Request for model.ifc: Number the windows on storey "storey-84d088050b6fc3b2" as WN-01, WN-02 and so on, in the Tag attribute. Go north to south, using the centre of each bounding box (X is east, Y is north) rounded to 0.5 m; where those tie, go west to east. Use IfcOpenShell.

First a look at what the model holds.

```python
import ifcopenshell
import ifcopenshell.util.element
import ifcopenshell.util.placement

model = ifcopenshell.open("model.ifc")
print(model.schema)
storey = next(s for s in model.by_type("IfcBuildingStorey") if s.Name == "storey-84d088050b6fc3b2")
windows = [e for e in ifcopenshell.util.element.get_decomposition(storey) if e.is_a("IfcWindow")]
for e in sorted(windows, key=lambda e: e.id()):
    origin = ifcopenshell.util.placement.get_local_placement(e.ObjectPlacement)[:3, 3]
    print(e.id(), e.Tag, e.Name, origin.round(2) + 0.0, sep=" | ")
```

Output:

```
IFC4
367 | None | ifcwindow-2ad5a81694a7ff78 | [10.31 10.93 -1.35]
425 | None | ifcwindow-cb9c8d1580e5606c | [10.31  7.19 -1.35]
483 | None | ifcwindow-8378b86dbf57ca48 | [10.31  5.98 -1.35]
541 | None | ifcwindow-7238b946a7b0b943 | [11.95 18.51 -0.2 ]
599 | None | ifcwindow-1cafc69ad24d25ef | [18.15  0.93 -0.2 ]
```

```python
import ifcopenshell
import ifcopenshell.geom
import ifcopenshell.util.element
import ifcopenshell.util.shape

model = ifcopenshell.open("model.ifc")
settings = ifcopenshell.geom.settings()
settings.set("use-world-coords", True)


def centre(element):
    shape = ifcopenshell.geom.create_shape(settings, element)
    return ifcopenshell.util.shape.get_bbox_centroid(shape.geometry)


storey = next(s for s in model.by_type("IfcBuildingStorey") if s.Name == "storey-84d088050b6fc3b2")
windows = [e for e in ifcopenshell.util.element.get_decomposition(storey) if e.is_a("IfcWindow")]

# Insertion points can sit at a corner or the storey origin, so sort by the geometry (in metres).
centres = {e: centre(e) for e in windows}
windows.sort(key=lambda e: (-round(centres[e][1] / 0.5), centres[e][0]))

for i, e in enumerate(windows, start=1):
    number = f"WN-{i:02d}"
    e.Tag = number
    print(e.id(), number)

model.write("model_edited.ifc")
```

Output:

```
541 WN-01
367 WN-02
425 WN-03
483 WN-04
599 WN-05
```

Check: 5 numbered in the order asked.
